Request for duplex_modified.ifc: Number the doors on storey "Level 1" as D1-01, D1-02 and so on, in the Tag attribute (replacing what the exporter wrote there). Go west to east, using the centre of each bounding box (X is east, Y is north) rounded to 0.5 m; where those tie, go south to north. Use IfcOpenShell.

First a look at what the model holds.

```python
import ifcopenshell
import ifcopenshell.util.element
import ifcopenshell.util.placement

model = ifcopenshell.open("duplex_modified.ifc")
print(model.schema)
storey = next(s for s in model.by_type("IfcBuildingStorey") if s.Name == "Level 1")
doors = [e for e in ifcopenshell.util.element.get_decomposition(storey) if e.is_a("IfcDoor")]
for e in sorted(doors, key=lambda e: e.id()):
    origin = ifcopenshell.util.placement.get_local_placement(e.ObjectPlacement)[:3, 3]
    print(e.id(), e.Tag, e.Name, origin.round(2) + 0.0, sep=" | ")
```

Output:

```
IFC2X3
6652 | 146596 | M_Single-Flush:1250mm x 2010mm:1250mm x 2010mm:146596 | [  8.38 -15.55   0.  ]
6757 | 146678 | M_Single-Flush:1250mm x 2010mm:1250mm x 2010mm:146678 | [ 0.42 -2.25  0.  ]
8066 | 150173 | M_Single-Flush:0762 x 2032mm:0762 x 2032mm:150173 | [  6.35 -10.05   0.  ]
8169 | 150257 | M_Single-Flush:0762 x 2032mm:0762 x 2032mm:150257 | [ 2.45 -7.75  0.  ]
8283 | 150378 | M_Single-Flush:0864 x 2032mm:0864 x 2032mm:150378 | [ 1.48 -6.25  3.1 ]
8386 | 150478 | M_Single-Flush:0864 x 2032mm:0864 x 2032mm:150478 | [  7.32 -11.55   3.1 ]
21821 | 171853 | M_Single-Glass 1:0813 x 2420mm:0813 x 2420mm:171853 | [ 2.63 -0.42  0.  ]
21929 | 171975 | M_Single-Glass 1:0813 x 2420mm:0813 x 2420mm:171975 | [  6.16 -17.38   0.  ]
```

```python
import ifcopenshell
import ifcopenshell.geom
import ifcopenshell.util.element
import ifcopenshell.util.shape

model = ifcopenshell.open("duplex_modified.ifc")
settings = ifcopenshell.geom.settings()
settings.set("use-world-coords", True)


def centre(element):
    shape = ifcopenshell.geom.create_shape(settings, element)
    return ifcopenshell.util.shape.get_bbox_centroid(shape.geometry)


storey = next(s for s in model.by_type("IfcBuildingStorey") if s.Name == "Level 1")
doors = [e for e in ifcopenshell.util.element.get_decomposition(storey) if e.is_a("IfcDoor")]

# Insertion points can sit at a corner or the storey origin, so sort by the geometry (in metres).
centres = {e: centre(e) for e in doors}
doors.sort(key=lambda e: (round(centres[e][0] / 0.5), centres[e][1]))

for i, e in enumerate(doors, start=1):
    number = f"D1-{i:02d}"
    e.Tag = number
    print(e.id(), number)

model.write("duplex_modified_rev.ifc")
```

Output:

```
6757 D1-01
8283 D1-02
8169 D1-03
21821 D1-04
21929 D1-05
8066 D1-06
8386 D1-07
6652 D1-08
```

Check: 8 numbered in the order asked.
